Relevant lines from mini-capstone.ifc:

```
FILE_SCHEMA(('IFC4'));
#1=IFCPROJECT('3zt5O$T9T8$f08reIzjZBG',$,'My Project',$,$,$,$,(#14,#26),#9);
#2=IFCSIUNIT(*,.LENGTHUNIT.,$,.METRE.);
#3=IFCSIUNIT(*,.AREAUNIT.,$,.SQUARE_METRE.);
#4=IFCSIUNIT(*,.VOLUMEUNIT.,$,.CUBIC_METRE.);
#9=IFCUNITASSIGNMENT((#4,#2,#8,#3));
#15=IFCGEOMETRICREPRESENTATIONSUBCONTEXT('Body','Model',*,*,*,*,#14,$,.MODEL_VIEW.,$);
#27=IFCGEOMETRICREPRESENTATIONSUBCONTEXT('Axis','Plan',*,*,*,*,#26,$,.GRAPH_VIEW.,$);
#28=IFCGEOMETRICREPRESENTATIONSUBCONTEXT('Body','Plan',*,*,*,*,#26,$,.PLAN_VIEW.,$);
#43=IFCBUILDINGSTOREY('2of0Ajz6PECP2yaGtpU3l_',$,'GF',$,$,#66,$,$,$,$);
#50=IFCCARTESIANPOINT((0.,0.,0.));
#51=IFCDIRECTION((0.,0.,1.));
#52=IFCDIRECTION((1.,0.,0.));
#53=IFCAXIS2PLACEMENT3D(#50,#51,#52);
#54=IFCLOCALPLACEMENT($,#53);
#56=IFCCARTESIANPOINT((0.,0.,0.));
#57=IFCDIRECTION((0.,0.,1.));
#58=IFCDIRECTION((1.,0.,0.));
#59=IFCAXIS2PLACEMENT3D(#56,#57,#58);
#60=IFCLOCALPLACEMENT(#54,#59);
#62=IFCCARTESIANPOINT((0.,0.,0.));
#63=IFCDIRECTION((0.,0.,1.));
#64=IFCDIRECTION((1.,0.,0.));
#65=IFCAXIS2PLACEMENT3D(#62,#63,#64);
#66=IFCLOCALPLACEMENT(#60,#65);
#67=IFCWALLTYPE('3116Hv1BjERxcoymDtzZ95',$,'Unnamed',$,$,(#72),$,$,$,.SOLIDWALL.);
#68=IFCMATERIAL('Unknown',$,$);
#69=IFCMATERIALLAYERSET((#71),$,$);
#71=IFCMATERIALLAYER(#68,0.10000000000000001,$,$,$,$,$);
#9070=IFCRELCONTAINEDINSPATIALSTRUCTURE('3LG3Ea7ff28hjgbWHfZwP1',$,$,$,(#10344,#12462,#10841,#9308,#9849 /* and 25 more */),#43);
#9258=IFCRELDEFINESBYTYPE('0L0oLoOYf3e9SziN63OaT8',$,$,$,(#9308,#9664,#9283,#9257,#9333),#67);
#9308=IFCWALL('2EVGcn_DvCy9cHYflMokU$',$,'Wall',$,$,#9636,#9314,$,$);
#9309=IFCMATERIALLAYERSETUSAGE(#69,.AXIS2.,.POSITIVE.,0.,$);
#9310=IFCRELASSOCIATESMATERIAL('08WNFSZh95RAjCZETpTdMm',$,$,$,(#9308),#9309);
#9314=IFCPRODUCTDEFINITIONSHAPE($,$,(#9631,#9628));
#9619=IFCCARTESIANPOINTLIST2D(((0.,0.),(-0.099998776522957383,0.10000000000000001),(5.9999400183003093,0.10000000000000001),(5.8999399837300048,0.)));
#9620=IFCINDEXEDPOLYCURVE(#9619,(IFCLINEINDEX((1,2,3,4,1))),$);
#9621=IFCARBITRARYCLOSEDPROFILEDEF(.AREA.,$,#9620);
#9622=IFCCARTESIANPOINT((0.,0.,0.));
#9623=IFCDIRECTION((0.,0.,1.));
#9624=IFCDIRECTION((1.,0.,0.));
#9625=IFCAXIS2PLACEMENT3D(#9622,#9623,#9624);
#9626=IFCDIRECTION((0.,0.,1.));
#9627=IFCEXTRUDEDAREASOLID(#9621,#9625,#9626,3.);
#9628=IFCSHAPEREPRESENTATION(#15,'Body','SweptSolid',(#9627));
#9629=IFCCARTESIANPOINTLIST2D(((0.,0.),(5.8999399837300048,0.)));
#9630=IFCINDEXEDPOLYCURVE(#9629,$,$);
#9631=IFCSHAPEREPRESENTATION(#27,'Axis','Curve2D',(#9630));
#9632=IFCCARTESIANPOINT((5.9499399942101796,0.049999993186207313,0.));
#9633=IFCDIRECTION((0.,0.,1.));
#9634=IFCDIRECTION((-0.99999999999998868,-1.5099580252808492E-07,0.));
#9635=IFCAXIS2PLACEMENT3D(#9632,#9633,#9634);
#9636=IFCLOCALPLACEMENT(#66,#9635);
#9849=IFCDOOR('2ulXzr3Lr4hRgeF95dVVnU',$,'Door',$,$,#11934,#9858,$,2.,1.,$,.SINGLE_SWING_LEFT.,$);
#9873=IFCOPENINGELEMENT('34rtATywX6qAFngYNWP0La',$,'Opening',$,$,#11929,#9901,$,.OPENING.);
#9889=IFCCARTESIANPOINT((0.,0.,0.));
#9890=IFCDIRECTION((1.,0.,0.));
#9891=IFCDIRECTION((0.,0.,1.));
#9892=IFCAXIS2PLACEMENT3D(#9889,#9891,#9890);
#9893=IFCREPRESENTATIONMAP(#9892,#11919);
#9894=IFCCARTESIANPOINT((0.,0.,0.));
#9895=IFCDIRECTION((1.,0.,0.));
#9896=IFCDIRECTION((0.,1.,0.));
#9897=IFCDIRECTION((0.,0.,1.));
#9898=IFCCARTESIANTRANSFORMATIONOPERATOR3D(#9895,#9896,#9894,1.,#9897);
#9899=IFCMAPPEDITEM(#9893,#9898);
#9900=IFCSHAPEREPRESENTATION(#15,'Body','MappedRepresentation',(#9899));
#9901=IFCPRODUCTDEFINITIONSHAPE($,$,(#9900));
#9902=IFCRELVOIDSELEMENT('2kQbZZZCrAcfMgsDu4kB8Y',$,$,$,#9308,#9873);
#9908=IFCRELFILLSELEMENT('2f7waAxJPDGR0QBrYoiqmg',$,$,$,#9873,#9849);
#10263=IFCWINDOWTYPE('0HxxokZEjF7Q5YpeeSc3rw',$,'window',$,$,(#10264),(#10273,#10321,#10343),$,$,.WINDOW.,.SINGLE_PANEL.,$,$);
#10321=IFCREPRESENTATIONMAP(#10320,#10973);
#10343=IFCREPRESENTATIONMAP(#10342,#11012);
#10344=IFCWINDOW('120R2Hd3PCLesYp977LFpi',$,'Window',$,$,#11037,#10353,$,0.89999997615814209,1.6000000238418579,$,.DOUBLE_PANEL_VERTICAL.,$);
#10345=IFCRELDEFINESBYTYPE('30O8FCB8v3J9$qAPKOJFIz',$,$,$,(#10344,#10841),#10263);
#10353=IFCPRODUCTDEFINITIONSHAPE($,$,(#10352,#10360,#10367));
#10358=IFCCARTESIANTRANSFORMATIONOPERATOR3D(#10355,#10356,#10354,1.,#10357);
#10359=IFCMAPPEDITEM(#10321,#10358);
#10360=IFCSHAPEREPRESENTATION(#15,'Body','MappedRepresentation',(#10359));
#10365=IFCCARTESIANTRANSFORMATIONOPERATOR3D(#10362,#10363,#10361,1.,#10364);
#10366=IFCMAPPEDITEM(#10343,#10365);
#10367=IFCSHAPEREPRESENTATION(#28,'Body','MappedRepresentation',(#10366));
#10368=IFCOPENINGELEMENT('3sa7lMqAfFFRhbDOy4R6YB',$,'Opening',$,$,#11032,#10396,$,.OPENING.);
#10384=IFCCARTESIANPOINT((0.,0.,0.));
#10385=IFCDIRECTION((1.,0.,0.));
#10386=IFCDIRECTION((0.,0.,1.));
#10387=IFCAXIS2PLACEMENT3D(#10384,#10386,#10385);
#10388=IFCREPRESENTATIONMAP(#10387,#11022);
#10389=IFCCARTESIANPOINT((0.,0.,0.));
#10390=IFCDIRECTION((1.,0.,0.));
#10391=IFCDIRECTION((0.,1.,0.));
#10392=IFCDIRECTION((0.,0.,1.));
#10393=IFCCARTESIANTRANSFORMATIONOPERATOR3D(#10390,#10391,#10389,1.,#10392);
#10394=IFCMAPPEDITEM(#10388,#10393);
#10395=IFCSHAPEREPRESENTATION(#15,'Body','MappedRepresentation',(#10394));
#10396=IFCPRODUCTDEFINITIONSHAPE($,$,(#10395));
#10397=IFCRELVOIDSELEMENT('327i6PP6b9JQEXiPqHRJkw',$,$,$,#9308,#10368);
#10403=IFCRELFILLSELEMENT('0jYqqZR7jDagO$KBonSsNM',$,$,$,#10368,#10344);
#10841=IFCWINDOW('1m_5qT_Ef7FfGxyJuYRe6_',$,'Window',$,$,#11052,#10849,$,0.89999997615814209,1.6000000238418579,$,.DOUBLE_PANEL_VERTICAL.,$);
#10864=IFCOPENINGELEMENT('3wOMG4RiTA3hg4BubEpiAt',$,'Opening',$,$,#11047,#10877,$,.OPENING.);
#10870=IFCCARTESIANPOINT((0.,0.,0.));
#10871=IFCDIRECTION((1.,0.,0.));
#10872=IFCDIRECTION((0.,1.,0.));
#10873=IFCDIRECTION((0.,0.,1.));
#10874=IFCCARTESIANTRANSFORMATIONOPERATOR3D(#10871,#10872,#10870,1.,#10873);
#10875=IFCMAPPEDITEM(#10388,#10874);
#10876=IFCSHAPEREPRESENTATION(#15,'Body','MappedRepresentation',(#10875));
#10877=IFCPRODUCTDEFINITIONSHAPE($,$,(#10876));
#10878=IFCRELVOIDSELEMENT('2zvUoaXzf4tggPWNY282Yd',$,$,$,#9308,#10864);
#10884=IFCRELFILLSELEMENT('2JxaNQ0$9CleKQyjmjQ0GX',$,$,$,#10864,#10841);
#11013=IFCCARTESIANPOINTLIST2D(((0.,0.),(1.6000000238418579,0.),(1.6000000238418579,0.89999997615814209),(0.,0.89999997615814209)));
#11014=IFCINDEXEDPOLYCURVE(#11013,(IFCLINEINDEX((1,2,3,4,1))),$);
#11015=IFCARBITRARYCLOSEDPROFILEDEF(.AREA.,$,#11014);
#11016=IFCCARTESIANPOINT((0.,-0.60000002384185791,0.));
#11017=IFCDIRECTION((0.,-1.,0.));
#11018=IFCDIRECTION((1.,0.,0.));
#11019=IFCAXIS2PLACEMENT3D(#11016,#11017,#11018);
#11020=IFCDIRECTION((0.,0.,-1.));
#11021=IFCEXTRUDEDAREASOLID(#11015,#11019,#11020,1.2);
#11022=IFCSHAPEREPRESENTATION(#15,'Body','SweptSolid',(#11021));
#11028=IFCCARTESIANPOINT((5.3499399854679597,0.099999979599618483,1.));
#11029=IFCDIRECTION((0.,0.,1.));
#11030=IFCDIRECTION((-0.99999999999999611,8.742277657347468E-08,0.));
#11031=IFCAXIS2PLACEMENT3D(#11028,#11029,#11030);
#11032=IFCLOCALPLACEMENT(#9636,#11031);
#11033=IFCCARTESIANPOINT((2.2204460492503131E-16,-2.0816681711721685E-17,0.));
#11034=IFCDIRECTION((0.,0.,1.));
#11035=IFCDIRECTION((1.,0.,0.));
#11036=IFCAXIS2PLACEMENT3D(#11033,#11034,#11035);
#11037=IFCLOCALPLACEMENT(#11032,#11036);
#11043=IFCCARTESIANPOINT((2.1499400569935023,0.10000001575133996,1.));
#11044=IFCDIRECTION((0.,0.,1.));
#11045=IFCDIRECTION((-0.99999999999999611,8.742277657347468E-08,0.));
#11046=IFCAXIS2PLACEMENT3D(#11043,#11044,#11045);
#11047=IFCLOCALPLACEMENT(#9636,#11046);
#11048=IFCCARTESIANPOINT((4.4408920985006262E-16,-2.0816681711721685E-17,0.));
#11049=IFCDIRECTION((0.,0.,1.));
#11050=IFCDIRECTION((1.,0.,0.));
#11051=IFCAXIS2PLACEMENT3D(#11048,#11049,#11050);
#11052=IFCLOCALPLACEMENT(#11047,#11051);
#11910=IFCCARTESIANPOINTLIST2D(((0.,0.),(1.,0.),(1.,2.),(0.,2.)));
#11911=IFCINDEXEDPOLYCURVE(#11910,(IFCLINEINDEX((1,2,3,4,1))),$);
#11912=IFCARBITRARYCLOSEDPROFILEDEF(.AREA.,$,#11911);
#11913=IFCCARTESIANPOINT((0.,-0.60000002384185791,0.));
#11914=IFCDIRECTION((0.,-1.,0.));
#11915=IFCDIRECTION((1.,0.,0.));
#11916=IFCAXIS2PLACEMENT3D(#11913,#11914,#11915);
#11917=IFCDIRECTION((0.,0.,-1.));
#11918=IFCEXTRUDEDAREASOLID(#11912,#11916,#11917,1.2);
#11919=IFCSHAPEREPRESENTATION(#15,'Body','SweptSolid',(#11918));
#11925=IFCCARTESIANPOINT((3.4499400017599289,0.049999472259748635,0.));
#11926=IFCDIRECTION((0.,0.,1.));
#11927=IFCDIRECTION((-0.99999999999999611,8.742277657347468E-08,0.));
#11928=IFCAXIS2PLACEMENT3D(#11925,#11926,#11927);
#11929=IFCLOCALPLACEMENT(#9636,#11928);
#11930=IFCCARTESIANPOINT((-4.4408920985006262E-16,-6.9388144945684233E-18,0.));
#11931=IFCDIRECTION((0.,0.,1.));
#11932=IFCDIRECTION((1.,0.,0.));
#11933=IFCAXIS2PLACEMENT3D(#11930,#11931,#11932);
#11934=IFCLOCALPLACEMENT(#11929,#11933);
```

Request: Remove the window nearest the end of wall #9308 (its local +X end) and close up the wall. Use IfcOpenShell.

```python
import ifcopenshell
import ifcopenshell.api.feature
import ifcopenshell.api.root
import ifcopenshell.geom
import ifcopenshell.util.shape

model = ifcopenshell.open("mini-capstone.ifc")
settings = ifcopenshell.geom.settings()


def volume(element):
    """Net volume in cubic metres, openings subtracted."""
    shape = ifcopenshell.geom.create_shape(settings, element)
    return ifcopenshell.util.shape.get_volume(shape.geometry)


window = model.by_guid("120R2Hd3PCLesYp977LFpi")
opening = window.FillsVoids[0].RelatingOpeningElement
wall = opening.VoidsElements[0].RelatingBuildingElement
before = volume(wall)

ifcopenshell.api.root.remove_product(model, product=window)
ifcopenshell.api.feature.remove_feature(model, feature=opening)

after = volume(wall)

print(f"wall volume {before:.3f} -> {after:.3f} m3")

model.write("mini-capstone_rev.ifc")
```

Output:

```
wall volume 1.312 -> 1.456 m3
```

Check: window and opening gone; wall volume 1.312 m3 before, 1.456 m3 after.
